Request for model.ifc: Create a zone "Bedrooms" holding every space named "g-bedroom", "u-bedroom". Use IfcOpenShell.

First a look at what the model holds.

```python
import ifcopenshell

model = ifcopenshell.open("model.ifc")
print(model.schema)
seen = {}
for space in model.by_type("IfcSpace"):
    seen[space.LongName] = seen.get(space.LongName, 0) + 1
for name, count in sorted(seen.items(), key=str):
    print(count, "x", name)
print("zones:", [z.Name for z in model.by_type("IfcZone")][:20])
```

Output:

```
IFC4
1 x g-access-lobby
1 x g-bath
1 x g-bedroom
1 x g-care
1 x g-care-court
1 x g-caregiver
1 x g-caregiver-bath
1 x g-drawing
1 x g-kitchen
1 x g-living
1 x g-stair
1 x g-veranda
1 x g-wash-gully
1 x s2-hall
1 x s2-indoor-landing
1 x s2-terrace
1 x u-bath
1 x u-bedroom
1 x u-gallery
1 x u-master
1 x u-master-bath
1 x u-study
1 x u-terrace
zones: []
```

```python
import ifcopenshell
import ifcopenshell.api.group
import ifcopenshell.api.root

model = ifcopenshell.open("model.ifc")

names = {"g-bedroom", "u-bedroom"}
spaces = [s for s in model.by_type("IfcSpace") if s.LongName in names]

zone = ifcopenshell.api.root.create_entity(model, ifc_class="IfcZone", name="Bedrooms")
ifcopenshell.api.group.assign_group(model, products=spaces, group=zone)
print(len(spaces), "spaces in", zone.Name)

model.write("model_rev.ifc")
```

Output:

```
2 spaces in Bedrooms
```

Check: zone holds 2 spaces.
